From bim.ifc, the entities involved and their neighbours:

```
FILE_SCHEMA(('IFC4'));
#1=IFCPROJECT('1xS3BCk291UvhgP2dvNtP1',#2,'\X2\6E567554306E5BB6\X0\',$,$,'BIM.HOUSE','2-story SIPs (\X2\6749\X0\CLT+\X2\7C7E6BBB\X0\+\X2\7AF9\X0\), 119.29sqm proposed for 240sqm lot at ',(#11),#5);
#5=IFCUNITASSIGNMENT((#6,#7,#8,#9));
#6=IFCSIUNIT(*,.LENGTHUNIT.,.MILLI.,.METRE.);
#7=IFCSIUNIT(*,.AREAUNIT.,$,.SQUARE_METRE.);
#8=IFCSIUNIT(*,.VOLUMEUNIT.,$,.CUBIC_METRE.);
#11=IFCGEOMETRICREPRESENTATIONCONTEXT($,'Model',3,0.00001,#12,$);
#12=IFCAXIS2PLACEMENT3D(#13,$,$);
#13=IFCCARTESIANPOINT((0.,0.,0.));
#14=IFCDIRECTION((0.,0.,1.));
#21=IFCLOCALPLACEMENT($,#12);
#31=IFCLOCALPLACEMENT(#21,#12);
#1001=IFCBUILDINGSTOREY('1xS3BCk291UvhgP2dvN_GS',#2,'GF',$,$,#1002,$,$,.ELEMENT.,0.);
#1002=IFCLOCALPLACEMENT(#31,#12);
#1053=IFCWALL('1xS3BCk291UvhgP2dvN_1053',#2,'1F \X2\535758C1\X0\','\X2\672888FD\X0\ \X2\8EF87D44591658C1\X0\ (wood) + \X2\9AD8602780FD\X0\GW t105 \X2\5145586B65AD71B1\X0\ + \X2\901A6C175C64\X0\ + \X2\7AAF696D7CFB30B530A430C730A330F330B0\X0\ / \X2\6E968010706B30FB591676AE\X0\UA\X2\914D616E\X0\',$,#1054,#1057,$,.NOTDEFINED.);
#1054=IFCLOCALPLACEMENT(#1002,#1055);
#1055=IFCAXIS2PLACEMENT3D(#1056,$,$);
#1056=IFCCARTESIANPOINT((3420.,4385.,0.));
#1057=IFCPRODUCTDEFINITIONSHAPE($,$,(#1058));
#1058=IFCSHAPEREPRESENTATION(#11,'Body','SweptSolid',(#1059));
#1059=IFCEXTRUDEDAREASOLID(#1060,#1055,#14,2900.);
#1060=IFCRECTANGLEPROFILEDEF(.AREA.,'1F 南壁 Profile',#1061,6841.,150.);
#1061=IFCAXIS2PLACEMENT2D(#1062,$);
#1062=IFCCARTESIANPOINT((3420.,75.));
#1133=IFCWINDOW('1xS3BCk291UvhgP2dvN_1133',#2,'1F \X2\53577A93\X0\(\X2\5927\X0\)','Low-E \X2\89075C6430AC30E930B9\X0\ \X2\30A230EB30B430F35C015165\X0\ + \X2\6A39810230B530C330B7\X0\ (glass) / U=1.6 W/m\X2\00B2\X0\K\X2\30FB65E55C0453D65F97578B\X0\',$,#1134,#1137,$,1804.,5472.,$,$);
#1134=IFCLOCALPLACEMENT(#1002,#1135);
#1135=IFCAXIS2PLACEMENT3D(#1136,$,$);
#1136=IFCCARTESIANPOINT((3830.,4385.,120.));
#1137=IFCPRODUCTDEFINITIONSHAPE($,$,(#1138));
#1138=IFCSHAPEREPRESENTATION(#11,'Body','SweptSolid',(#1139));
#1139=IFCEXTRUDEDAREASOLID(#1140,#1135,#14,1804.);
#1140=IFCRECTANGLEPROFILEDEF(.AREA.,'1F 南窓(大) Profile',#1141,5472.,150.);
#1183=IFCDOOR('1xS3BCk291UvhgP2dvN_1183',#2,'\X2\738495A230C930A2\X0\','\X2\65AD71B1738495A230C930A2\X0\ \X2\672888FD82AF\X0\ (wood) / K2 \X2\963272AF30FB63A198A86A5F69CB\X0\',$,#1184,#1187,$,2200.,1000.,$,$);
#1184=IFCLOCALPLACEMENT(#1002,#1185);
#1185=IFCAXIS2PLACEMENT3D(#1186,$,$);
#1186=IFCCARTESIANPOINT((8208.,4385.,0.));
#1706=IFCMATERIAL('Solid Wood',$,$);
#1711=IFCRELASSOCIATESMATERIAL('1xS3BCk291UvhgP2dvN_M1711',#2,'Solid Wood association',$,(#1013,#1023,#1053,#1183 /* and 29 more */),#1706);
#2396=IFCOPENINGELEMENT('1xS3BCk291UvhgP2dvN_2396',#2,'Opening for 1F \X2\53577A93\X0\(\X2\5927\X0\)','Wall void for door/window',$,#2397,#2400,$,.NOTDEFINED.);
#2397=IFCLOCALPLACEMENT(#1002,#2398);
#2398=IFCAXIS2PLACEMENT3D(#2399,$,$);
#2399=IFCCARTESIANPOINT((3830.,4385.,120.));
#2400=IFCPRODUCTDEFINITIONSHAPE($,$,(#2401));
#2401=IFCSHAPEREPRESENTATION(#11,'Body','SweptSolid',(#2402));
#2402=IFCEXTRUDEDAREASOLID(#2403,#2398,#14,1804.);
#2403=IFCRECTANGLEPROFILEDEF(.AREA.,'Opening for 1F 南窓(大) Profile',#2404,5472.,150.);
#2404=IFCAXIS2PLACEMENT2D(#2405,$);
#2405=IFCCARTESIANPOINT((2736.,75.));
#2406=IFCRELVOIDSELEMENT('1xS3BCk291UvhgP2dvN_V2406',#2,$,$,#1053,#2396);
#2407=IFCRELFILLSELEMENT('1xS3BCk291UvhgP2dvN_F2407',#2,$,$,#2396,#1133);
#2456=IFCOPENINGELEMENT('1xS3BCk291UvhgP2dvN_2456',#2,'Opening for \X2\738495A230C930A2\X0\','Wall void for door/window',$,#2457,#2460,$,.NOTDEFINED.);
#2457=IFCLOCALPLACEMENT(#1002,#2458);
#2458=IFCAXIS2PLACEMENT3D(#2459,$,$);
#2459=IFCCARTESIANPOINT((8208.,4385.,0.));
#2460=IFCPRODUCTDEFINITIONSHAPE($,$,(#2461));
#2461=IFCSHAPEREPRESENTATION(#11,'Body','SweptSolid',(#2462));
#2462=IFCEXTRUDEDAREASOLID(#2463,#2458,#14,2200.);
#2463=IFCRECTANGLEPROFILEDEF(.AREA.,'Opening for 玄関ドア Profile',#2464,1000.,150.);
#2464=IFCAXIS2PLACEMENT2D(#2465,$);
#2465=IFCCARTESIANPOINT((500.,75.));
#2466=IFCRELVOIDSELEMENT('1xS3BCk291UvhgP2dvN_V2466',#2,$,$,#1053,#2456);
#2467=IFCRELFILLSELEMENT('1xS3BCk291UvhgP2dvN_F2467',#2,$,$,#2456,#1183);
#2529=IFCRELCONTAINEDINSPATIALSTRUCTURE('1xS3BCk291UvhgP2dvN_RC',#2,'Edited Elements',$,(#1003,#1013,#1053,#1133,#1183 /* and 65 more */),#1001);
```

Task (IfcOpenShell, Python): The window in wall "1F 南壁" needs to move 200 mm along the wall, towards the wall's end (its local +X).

```python
import ifcopenshell
import ifcopenshell.api.geometry
import ifcopenshell.util.placement
import ifcopenshell.util.unit

model = ifcopenshell.open("bim.ifc")
unit_scale = ifcopenshell.util.unit.calculate_unit_scale(model)

window = model.by_id(1133)
opening = window.FillsVoids[0].RelatingOpeningElement
wall = opening.VoidsElements[0].RelatingBuildingElement

wall_matrix = ifcopenshell.util.placement.get_local_placement(wall.ObjectPlacement)
shift = wall_matrix[:3, 0] * 0.2 / unit_scale
before = ifcopenshell.util.placement.get_local_placement(window.ObjectPlacement)[:3, 3].copy()

# The window is not placed relative to its opening, so move both.
for product in (opening, window):
    matrix = ifcopenshell.util.placement.get_local_placement(product.ObjectPlacement)
    matrix[:3, 3] += shift
    ifcopenshell.api.geometry.edit_object_placement(model, product=product, matrix=matrix, is_si=False)

after = ifcopenshell.util.placement.get_local_placement(window.ObjectPlacement)[:3, 3]
print("window moved by", (after - before).round(3) + 0.0)

model.write("bim_updated.ifc")
```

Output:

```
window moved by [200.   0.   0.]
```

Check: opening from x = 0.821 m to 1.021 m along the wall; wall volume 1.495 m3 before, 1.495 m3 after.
